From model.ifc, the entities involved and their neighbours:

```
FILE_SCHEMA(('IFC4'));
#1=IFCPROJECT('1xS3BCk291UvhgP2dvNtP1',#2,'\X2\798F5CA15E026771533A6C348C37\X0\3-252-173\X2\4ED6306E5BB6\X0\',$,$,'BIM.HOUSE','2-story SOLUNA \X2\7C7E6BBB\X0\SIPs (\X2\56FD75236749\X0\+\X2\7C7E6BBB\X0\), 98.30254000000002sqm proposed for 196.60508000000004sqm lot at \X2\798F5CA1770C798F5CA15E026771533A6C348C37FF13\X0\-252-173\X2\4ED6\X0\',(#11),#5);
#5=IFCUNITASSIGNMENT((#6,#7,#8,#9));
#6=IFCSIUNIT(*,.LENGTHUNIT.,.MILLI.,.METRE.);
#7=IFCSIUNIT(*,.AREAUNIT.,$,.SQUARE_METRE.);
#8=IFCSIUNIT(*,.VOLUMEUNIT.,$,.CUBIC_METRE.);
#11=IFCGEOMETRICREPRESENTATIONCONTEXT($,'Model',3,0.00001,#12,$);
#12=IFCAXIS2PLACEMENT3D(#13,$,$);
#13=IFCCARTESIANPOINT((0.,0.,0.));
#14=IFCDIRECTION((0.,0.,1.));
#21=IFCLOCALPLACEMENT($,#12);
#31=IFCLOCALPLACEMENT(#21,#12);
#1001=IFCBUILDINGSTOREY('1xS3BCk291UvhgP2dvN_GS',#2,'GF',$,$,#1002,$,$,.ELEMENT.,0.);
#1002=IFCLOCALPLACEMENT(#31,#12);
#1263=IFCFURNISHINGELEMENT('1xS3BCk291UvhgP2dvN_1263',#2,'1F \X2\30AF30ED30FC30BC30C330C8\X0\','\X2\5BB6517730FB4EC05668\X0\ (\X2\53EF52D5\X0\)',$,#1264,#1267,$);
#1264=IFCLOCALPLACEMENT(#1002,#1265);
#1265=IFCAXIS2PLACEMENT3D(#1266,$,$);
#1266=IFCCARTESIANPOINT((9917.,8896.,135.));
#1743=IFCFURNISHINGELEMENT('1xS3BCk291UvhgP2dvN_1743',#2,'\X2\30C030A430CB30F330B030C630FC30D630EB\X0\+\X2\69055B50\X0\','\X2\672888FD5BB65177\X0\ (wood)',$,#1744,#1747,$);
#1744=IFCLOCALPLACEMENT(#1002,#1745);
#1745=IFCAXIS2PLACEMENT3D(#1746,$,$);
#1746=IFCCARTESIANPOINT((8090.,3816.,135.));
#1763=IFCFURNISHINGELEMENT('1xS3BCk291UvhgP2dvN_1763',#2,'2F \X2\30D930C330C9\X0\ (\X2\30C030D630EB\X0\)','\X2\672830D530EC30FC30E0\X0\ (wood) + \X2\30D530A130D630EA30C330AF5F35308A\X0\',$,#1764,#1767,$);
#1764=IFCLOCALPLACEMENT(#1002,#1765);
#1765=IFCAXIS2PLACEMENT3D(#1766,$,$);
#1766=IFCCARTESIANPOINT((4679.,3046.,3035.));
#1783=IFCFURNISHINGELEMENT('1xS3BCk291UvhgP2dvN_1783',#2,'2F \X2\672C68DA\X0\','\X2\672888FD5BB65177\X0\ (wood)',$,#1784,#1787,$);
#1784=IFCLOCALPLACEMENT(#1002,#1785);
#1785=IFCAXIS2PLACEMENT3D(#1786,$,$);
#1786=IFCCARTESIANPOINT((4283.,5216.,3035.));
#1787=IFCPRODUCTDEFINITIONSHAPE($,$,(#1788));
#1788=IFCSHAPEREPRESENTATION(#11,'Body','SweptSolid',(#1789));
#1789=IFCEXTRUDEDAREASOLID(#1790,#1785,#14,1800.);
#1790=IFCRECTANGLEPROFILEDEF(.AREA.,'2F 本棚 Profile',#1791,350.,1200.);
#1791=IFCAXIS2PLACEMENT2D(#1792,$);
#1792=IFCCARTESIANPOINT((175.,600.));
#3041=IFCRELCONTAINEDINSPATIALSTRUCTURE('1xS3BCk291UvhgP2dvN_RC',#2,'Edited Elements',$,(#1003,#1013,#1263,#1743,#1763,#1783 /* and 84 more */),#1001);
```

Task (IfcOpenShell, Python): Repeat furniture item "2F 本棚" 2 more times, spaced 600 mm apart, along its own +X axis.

```python
import ifcopenshell
import ifcopenshell.api.geometry
import ifcopenshell.api.root
import ifcopenshell.util.element
import ifcopenshell.util.placement
import ifcopenshell.util.unit

model = ifcopenshell.open("model.ifc")
unit_scale = ifcopenshell.util.unit.calculate_unit_scale(model)


def reuse_history(source, copy):
    """copy_class also copies each property set's owner history, people and application; keep the originals."""
    for rel in copy.IsDefinedBy:
        if rel.is_a("IfcRelDefinesByProperties") and (history := rel.RelatingPropertyDefinition.OwnerHistory):
            rel.RelatingPropertyDefinition.OwnerHistory = source.OwnerHistory
            ifcopenshell.util.element.remove_deep2(model, history)


source = model.by_id(1783)
base = ifcopenshell.util.placement.get_local_placement(source.ObjectPlacement)
step = base[:3, 0] * 0.6 / unit_scale

for i in range(1, 3):
    copy = ifcopenshell.api.root.copy_class(model, product=source)
    copy.Representation = ifcopenshell.util.element.copy_deep(
        model, source.Representation, exclude=["IfcGeometricRepresentationContext", "IfcRepresentationMap"]
    )
    reuse_history(source, copy)
    matrix = base.copy()
    matrix[:3, 3] += i * step
    print("added at", matrix[:3, 3].round(3) + 0.0)
    ifcopenshell.api.geometry.edit_object_placement(model, product=copy, matrix=matrix, is_si=False)

model.write("model-out.ifc")
```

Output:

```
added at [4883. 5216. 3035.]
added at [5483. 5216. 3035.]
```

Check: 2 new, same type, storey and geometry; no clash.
